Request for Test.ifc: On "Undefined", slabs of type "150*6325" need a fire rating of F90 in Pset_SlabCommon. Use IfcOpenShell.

First a look at what the model holds.

```python
import ifcopenshell
import ifcopenshell.util.element

model = ifcopenshell.open("Test.ifc")
print(model.schema)
storey = next(s for s in model.by_type("IfcBuildingStorey") if s.Name == "Undefined")
slabs = [e for e in ifcopenshell.util.element.get_decomposition(storey) if e.is_a("IfcSlab")]
seen = {}
for e in slabs:
    element_type = ifcopenshell.util.element.get_type(e)
    key = (element_type.Name if element_type != e and element_type else None, ifcopenshell.util.element.get_pset(e, "Pset_SlabCommon", "FireRating"))
    seen[key] = seen.get(key, 0) + 1
for (name, value), count in sorted(seen.items(), key=str):
    print(count, "x", name, "|", value)
```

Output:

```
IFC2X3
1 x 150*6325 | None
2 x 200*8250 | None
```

```python
import ifcopenshell
import ifcopenshell.api.pset
import ifcopenshell.util.element

model = ifcopenshell.open("Test.ifc")

storey = next(s for s in model.by_type("IfcBuildingStorey") if s.Name == "Undefined")
slabs = [e for e in ifcopenshell.util.element.get_decomposition(storey) if e.is_a("IfcSlab")]

count = 0
for e in slabs:
    element_type = ifcopenshell.util.element.get_type(e)
    if element_type in (None, e) or element_type.Name != "150*6325":
        continue
    found = ifcopenshell.util.element.get_pset(e, "Pset_SlabCommon", should_inherit=False)
    if found:
        pset = model.by_id(found["id"])
        if len(ifcopenshell.util.element.get_elements_by_pset(pset)) > 1:
            pset = ifcopenshell.api.pset.unshare_pset(model, products=[e], pset=pset)[0]
    else:
        pset = ifcopenshell.api.pset.add_pset(model, product=e, name="Pset_SlabCommon")
    ifcopenshell.api.pset.edit_pset(model, pset=pset, properties={"FireRating": "F90"})
    count += 1

print(count, "slabs updated")

model.write("Test-out.ifc")
```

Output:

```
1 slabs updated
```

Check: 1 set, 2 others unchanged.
